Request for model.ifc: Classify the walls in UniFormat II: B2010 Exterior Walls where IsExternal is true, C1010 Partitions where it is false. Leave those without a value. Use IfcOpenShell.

First a look at what the model holds.

```python
import ifcopenshell
import ifcopenshell.util.element

model = ifcopenshell.open("model.ifc")
print(model.schema)
print("classifications:", [c.Name for c in model.by_type("IfcClassification")])
values = [ifcopenshell.util.element.get_pset(e, "Pset_WallCommon", "IsExternal") for e in model.by_type("IfcWall")]
for value in (True, False, None):
    print("IsExternal", value, values.count(value))
```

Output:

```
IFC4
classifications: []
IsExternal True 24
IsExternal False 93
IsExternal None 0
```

```python
import ifcopenshell
import ifcopenshell.api.classification
import ifcopenshell.util.element

model = ifcopenshell.open("model.ifc")

system = ifcopenshell.api.classification.add_classification(model, classification="UniFormat II")

walls = model.by_type("IfcWall")
external = {e: ifcopenshell.util.element.get_pset(e, "Pset_WallCommon", "IsExternal") for e in walls}
for flag, code, name in ((True, "B2010", "Exterior Walls"), (False, "C1010", "Partitions")):
    products = [e for e in walls if external[e] is flag]
    ifcopenshell.api.classification.add_reference(
        model, products=products, classification=system, identification=code, name=name
    )
    print(code, len(products))

model.write("model_v2.ifc")
```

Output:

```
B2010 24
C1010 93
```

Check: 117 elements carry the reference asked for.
